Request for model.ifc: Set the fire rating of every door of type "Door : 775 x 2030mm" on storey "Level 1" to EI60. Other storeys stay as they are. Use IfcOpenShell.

First a look at what the model holds.

```python
import ifcopenshell
import ifcopenshell.util.element

model = ifcopenshell.open("model.ifc")
print(model.schema)
storey = next(s for s in model.by_type("IfcBuildingStorey") if s.Name == "Level 1")
doors = [e for e in ifcopenshell.util.element.get_decomposition(storey) if e.is_a("IfcDoor")]
seen = {}
for e in doors:
    element_type = ifcopenshell.util.element.get_type(e)
    key = (element_type.Name if element_type != e and element_type else None, ifcopenshell.util.element.get_pset(e, "Pset_DoorCommon", "FireRating"))
    seen[key] = seen.get(key, 0) + 1
for (name, value), count in sorted(seen.items(), key=str):
    print(count, "x", name, "|", value)
```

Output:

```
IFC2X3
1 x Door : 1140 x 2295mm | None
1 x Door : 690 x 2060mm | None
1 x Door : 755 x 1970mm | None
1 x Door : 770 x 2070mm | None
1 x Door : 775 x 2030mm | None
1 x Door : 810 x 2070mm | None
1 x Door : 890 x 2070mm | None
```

```python
import ifcopenshell
import ifcopenshell.api.pset
import ifcopenshell.util.element

model = ifcopenshell.open("model.ifc")

storey = next(s for s in model.by_type("IfcBuildingStorey") if s.Name == "Level 1")
doors = [e for e in ifcopenshell.util.element.get_decomposition(storey) if e.is_a("IfcDoor")]

count = 0
for e in doors:
    element_type = ifcopenshell.util.element.get_type(e)
    if element_type in (None, e) or element_type.Name != "Door : 775 x 2030mm":
        continue
    # add_pset returns the element's existing set when there is one.
    pset = ifcopenshell.api.pset.add_pset(model, product=e, name="Pset_DoorCommon")
    ifcopenshell.api.pset.edit_pset(model, pset=pset, properties={"FireRating": "EI60"})
    count += 1

print(count, "doors updated")

model.write("model-out.ifc")
```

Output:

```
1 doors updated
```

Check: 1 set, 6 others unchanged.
